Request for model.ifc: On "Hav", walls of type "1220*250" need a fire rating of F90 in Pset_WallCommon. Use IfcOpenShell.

First a look at what the model holds.

```python
import ifcopenshell
import ifcopenshell.util.element

model = ifcopenshell.open("model.ifc")
print(model.schema)
storey = next(s for s in model.by_type("IfcBuildingStorey") if s.Name == "Hav")
walls = [e for e in ifcopenshell.util.element.get_decomposition(storey) if e.is_a("IfcWall")]
seen = {}
for e in walls:
    element_type = ifcopenshell.util.element.get_type(e)
    key = (element_type.Name if element_type != e and element_type else None, ifcopenshell.util.element.get_pset(e, "Pset_WallCommon", "FireRating"))
    seen[key] = seen.get(key, 0) + 1
for (name, value), count in sorted(seen.items(), key=str):
    print(count, "x", name, "|", value)
```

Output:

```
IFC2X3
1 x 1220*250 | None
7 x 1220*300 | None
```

```python
import ifcopenshell
import ifcopenshell.api.pset
import ifcopenshell.util.element

model = ifcopenshell.open("model.ifc")

storey = next(s for s in model.by_type("IfcBuildingStorey") if s.Name == "Hav")
walls = [e for e in ifcopenshell.util.element.get_decomposition(storey) if e.is_a("IfcWall")]

count = 0
for e in walls:
    element_type = ifcopenshell.util.element.get_type(e)
    if element_type in (None, e) or element_type.Name != "1220*250":
        continue
    found = ifcopenshell.util.element.get_pset(e, "Pset_WallCommon", should_inherit=False)
    if found:
        pset = model.by_id(found["id"])
        if len(ifcopenshell.util.element.get_elements_by_pset(pset)) > 1:
            pset = ifcopenshell.api.pset.unshare_pset(model, products=[e], pset=pset)[0]
    else:
        pset = ifcopenshell.api.pset.add_pset(model, product=e, name="Pset_WallCommon")
    ifcopenshell.api.pset.edit_pset(model, pset=pset, properties={"FireRating": "F90"})
    count += 1

print(count, "walls updated")

model.write("model_edited.ifc")
```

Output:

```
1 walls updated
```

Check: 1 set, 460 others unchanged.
